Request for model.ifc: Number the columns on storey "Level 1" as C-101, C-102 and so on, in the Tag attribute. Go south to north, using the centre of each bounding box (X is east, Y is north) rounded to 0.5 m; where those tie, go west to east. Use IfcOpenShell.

First a look at what the model holds.

```python
import ifcopenshell
import ifcopenshell.util.element
import ifcopenshell.util.placement

model = ifcopenshell.open("model.ifc")
print(model.schema)
storey = next(s for s in model.by_type("IfcBuildingStorey") if s.Name == "Level 1")
columns = [e for e in ifcopenshell.util.element.get_decomposition(storey) if e.is_a("IfcColumn")]
for e in sorted(columns, key=lambda e: e.id()):
    origin = ifcopenshell.util.placement.get_local_placement(e.ObjectPlacement)[:3, 3]
    print(e.id(), e.Tag, e.Name, origin.round(2) + 0.0, sep=" | ")
```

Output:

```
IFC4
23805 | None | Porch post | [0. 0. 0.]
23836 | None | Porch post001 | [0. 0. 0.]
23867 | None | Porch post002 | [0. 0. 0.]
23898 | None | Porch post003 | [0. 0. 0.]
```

```python
import ifcopenshell
import ifcopenshell.geom
import ifcopenshell.util.element
import ifcopenshell.util.shape

model = ifcopenshell.open("model.ifc")
settings = ifcopenshell.geom.settings()
settings.set("use-world-coords", True)


def centre(element):
    shape = ifcopenshell.geom.create_shape(settings, element)
    return ifcopenshell.util.shape.get_bbox_centroid(shape.geometry)


storey = next(s for s in model.by_type("IfcBuildingStorey") if s.Name == "Level 1")
columns = [e for e in ifcopenshell.util.element.get_decomposition(storey) if e.is_a("IfcColumn")]

# Insertion points can sit at a corner or the storey origin, so sort by the geometry (in metres).
centres = {e: centre(e) for e in columns}
columns.sort(key=lambda e: (round(centres[e][1] / 0.5), centres[e][0]))

for i, e in enumerate(columns, start=1):
    number = f"C-1{i:02d}"
    e.Tag = number
    print(e.id(), number)

model.write("model_rev.ifc")
```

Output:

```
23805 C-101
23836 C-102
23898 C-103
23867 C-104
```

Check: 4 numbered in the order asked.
